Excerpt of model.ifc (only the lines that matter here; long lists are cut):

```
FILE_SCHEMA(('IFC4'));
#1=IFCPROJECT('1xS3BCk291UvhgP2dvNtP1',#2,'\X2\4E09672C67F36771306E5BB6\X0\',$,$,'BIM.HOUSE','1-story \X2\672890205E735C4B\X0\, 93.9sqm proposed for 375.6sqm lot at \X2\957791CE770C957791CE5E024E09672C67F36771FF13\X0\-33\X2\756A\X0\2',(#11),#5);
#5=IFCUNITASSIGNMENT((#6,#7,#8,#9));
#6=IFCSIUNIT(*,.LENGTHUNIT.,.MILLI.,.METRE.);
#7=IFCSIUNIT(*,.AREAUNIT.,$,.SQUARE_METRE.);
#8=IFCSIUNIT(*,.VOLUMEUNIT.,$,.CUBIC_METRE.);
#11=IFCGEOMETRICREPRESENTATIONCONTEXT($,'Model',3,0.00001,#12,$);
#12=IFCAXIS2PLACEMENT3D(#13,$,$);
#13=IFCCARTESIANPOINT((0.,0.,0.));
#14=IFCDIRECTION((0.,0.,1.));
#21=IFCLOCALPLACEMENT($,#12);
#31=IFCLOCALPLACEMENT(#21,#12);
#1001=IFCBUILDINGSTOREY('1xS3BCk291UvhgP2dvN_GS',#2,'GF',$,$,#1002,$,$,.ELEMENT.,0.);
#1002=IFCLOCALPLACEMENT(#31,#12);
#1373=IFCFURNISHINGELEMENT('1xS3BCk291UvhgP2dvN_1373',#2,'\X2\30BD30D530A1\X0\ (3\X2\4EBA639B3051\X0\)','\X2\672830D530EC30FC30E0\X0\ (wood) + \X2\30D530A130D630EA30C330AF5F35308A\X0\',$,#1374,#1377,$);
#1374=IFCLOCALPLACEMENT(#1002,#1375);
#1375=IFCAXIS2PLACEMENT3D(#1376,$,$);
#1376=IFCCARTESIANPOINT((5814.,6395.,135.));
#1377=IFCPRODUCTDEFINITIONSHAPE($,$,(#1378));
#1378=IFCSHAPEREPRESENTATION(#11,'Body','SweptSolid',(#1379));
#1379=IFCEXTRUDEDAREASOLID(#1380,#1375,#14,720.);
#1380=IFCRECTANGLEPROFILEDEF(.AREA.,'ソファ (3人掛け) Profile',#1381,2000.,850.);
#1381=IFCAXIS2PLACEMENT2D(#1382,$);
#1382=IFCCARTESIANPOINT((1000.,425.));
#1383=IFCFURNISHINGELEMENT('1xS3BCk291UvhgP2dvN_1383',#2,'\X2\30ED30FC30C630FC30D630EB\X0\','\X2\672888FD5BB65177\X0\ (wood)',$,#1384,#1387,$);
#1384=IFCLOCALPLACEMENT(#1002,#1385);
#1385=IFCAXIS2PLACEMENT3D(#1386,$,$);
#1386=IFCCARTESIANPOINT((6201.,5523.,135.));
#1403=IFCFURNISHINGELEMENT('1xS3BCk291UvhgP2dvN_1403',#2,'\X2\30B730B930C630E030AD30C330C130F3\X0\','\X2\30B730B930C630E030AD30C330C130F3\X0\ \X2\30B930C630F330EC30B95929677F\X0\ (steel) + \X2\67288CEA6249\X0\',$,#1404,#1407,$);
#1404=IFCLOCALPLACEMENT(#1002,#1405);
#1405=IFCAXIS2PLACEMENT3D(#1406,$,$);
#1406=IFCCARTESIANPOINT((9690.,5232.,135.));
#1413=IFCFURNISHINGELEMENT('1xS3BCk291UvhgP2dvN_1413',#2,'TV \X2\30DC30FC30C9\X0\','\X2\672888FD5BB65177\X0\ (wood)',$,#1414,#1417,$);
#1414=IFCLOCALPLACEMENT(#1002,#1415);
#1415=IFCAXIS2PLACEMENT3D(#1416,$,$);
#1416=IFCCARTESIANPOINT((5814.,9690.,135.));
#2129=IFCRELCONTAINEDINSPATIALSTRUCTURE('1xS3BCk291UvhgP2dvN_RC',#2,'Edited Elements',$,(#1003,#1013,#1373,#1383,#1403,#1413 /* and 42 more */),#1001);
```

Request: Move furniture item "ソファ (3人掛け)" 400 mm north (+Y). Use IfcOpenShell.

```python
import ifcopenshell
import ifcopenshell.api.geometry
import ifcopenshell.util.placement

model = ifcopenshell.open("model.ifc")

item = model.by_id(1373)
matrix = ifcopenshell.util.placement.get_local_placement(item.ObjectPlacement)
matrix[1, 3] += 400.0
ifcopenshell.api.geometry.edit_object_placement(model, product=item, matrix=matrix, is_si=False)

print(ifcopenshell.util.placement.get_local_placement(item.ObjectPlacement).round(3) + 0.0)

model.write("model-out.ifc")
```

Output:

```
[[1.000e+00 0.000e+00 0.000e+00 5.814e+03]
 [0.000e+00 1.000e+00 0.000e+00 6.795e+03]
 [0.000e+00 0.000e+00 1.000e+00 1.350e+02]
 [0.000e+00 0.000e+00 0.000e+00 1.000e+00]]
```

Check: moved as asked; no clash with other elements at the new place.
